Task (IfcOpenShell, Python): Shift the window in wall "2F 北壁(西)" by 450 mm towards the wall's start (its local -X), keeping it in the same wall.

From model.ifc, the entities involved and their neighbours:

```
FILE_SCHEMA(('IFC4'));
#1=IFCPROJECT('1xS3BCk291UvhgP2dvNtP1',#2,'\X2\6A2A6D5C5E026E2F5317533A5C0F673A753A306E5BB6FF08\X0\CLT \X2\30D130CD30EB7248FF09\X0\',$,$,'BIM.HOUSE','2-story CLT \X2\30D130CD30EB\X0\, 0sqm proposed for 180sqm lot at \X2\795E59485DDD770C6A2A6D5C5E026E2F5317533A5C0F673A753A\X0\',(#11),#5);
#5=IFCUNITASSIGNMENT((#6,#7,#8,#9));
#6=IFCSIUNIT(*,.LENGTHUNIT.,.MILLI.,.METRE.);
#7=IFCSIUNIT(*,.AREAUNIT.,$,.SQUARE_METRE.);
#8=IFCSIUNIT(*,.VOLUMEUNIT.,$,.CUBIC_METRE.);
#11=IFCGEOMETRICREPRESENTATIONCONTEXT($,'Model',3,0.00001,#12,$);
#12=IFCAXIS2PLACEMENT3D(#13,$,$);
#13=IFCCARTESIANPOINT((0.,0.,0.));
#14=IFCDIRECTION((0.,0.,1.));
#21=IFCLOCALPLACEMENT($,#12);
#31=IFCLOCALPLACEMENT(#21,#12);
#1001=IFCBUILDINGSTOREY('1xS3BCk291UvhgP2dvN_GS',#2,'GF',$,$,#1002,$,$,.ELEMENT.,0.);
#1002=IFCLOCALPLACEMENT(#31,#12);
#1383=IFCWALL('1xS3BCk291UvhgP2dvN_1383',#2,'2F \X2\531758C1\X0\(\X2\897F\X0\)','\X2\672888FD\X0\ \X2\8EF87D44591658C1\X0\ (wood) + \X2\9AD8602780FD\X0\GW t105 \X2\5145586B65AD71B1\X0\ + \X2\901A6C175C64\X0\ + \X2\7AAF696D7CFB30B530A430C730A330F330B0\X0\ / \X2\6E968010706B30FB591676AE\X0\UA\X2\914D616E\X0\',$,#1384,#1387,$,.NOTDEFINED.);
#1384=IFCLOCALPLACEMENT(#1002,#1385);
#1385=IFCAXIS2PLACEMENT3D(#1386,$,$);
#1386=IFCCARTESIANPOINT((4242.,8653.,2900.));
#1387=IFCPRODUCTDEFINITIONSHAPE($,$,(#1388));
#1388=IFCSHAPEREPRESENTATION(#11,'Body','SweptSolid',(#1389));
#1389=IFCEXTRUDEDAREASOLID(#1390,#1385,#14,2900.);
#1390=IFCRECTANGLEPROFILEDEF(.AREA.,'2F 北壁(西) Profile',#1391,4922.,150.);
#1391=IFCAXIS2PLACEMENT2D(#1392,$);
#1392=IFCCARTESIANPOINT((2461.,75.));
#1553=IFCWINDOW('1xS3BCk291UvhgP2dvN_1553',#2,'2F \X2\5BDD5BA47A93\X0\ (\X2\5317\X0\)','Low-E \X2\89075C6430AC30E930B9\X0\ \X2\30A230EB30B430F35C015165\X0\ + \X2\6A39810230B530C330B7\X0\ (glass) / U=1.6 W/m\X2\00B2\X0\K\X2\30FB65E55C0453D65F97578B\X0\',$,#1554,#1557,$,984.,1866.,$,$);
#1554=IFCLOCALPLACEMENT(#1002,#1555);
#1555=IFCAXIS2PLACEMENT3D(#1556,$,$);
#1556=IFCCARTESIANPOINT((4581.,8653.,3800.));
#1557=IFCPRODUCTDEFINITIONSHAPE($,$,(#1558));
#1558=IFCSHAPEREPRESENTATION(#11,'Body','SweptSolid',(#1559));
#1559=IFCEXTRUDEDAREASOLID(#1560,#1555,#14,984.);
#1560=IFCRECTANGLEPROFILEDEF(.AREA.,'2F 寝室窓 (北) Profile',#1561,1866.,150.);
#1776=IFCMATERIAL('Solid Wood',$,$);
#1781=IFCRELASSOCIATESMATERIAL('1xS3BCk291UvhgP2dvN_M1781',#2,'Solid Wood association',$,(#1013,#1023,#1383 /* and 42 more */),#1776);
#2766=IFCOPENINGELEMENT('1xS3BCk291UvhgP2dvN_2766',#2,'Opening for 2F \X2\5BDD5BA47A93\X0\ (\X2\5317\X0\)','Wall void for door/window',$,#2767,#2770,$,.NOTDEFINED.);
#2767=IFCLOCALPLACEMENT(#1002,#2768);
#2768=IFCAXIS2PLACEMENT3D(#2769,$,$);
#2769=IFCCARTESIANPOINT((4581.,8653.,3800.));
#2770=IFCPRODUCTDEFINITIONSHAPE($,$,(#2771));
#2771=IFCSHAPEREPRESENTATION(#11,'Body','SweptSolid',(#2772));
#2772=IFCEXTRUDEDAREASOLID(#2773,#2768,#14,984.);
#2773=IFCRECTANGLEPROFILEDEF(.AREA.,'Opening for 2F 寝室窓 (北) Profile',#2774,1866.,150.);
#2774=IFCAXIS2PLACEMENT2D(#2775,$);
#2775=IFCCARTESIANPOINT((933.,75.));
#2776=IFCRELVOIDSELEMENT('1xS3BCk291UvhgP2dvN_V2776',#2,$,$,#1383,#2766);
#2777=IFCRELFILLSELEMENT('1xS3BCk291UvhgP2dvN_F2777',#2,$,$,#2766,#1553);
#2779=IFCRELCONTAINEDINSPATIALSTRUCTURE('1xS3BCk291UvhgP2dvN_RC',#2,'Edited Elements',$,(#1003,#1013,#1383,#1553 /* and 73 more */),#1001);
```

```python
import ifcopenshell
import ifcopenshell.api.geometry
import ifcopenshell.util.placement
import ifcopenshell.util.unit

model = ifcopenshell.open("model.ifc")
unit_scale = ifcopenshell.util.unit.calculate_unit_scale(model)

window = model.by_id(1553)
opening = window.FillsVoids[0].RelatingOpeningElement
wall = opening.VoidsElements[0].RelatingBuildingElement

wall_matrix = ifcopenshell.util.placement.get_local_placement(wall.ObjectPlacement)
shift = wall_matrix[:3, 0] * -0.45 / unit_scale
before = ifcopenshell.util.placement.get_local_placement(window.ObjectPlacement)[:3, 3].copy()

# The window is not placed relative to its opening, so move both.
for product in (opening, window):
    matrix = ifcopenshell.util.placement.get_local_placement(product.ObjectPlacement)
    matrix[:3, 3] += shift
    ifcopenshell.api.geometry.edit_object_placement(model, product=product, matrix=matrix, is_si=False)

after = ifcopenshell.util.placement.get_local_placement(window.ObjectPlacement)[:3, 3]
print("window moved by", (after - before).round(3) + 0.0)

model.write("model_updated.ifc")
```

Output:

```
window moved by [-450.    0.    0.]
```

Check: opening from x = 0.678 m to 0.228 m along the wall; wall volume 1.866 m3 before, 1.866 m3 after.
